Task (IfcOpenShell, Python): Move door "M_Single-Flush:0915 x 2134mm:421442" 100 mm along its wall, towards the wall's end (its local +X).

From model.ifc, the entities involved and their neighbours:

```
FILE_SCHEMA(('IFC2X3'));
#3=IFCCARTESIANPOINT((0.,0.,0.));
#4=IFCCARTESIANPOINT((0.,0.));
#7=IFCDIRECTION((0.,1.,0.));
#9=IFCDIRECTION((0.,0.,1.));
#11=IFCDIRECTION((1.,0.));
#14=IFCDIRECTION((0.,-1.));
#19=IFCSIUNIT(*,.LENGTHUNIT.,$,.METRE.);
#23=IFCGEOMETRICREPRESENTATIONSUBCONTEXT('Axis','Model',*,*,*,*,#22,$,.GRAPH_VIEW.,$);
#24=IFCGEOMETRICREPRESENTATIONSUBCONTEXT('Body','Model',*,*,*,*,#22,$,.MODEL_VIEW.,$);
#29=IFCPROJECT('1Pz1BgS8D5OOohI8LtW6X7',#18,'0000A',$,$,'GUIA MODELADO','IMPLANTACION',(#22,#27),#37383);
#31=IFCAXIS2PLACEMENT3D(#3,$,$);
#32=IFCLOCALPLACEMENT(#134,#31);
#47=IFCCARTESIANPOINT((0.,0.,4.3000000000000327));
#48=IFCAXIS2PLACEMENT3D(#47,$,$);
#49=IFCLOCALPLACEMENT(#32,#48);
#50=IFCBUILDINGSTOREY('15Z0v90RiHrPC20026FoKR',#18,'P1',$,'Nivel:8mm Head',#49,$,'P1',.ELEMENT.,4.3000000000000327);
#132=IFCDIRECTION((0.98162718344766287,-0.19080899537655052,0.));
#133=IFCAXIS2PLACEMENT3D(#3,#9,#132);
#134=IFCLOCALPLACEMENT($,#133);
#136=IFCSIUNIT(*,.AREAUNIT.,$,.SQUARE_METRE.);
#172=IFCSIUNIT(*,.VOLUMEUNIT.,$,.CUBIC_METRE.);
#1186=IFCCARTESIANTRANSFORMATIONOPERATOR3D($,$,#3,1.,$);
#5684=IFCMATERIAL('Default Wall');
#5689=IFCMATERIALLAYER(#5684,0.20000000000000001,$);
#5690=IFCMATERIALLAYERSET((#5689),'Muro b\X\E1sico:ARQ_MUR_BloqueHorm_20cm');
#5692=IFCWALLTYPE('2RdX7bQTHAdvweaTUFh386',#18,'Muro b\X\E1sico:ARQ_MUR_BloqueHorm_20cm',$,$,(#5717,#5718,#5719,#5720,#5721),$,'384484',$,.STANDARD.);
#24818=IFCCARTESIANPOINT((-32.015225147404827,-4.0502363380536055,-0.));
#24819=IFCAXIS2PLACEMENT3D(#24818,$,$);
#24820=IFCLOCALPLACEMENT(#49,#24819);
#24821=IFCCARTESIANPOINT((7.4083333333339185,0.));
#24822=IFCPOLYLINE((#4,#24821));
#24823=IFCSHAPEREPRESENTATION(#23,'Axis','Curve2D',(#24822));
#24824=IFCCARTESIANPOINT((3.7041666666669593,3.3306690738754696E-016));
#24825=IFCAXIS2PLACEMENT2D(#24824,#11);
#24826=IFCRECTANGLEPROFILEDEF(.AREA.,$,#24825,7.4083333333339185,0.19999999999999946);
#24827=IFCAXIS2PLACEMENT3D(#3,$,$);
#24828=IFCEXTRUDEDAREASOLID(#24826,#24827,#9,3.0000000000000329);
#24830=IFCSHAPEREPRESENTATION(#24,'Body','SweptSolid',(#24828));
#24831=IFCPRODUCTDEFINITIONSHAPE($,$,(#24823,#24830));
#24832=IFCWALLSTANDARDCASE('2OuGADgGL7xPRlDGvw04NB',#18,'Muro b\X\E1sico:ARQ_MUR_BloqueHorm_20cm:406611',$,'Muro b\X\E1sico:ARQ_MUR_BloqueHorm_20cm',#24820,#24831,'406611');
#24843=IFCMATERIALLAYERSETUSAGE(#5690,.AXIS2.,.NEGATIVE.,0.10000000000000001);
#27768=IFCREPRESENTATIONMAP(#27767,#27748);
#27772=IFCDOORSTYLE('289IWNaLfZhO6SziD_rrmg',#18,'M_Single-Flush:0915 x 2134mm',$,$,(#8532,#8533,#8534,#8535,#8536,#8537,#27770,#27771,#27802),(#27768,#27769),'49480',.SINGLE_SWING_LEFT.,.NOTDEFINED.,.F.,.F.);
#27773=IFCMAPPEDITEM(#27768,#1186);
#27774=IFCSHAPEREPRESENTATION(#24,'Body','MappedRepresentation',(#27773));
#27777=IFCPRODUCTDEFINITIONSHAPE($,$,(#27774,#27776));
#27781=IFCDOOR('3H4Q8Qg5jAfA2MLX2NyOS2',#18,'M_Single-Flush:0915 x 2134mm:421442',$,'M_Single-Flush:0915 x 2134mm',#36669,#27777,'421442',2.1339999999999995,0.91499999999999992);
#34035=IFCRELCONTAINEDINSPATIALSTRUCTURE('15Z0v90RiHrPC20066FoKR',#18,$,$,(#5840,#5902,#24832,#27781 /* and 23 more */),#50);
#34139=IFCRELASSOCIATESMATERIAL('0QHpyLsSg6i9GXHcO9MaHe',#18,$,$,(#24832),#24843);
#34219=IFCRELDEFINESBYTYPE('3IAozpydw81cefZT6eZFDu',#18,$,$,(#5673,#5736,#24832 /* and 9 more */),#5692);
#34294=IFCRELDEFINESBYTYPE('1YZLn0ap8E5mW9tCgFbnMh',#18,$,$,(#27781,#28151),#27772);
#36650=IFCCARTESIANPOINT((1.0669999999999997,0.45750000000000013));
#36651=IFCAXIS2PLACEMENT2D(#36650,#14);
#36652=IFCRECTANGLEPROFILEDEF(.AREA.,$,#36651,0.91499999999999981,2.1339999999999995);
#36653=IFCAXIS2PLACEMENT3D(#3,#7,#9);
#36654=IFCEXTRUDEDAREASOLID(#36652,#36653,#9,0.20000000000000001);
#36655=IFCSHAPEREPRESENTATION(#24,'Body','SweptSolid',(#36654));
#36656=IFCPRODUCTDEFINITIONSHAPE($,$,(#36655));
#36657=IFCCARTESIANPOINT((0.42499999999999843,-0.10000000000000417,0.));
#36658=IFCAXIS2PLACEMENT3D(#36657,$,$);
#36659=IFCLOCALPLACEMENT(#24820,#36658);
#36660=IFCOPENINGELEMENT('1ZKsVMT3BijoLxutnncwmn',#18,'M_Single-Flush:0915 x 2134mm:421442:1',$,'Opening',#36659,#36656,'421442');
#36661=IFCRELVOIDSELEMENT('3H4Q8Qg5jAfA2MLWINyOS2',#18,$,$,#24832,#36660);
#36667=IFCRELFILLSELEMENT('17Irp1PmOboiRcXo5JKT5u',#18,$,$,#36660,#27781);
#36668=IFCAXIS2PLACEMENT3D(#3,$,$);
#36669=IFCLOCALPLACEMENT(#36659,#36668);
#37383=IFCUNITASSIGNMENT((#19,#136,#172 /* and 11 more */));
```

```python
import ifcopenshell
import ifcopenshell.api.geometry
import ifcopenshell.util.placement

model = ifcopenshell.open("model.ifc")

door = model.by_guid("3H4Q8Qg5jAfA2MLX2NyOS2")
opening = door.FillsVoids[0].RelatingOpeningElement
wall = opening.VoidsElements[0].RelatingBuildingElement

wall_matrix = ifcopenshell.util.placement.get_local_placement(wall.ObjectPlacement)
shift = wall_matrix[:3, 0] * 0.1
before = ifcopenshell.util.placement.get_local_placement(door.ObjectPlacement)[:3, 3].copy()

# The door is placed relative to its opening, so it follows when the opening moves.
matrix = ifcopenshell.util.placement.get_local_placement(opening.ObjectPlacement)
matrix[:3, 3] += shift
ifcopenshell.api.geometry.edit_object_placement(
    model, product=opening, matrix=matrix, is_si=False, should_transform_children=True
)

after = ifcopenshell.util.placement.get_local_placement(door.ObjectPlacement)[:3, 3]
print("door moved by", (after - before).round(3) + 0.0)

model.write("model_rev.ifc")
```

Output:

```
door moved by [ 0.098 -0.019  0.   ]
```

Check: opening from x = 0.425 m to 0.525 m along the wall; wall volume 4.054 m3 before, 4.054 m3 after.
